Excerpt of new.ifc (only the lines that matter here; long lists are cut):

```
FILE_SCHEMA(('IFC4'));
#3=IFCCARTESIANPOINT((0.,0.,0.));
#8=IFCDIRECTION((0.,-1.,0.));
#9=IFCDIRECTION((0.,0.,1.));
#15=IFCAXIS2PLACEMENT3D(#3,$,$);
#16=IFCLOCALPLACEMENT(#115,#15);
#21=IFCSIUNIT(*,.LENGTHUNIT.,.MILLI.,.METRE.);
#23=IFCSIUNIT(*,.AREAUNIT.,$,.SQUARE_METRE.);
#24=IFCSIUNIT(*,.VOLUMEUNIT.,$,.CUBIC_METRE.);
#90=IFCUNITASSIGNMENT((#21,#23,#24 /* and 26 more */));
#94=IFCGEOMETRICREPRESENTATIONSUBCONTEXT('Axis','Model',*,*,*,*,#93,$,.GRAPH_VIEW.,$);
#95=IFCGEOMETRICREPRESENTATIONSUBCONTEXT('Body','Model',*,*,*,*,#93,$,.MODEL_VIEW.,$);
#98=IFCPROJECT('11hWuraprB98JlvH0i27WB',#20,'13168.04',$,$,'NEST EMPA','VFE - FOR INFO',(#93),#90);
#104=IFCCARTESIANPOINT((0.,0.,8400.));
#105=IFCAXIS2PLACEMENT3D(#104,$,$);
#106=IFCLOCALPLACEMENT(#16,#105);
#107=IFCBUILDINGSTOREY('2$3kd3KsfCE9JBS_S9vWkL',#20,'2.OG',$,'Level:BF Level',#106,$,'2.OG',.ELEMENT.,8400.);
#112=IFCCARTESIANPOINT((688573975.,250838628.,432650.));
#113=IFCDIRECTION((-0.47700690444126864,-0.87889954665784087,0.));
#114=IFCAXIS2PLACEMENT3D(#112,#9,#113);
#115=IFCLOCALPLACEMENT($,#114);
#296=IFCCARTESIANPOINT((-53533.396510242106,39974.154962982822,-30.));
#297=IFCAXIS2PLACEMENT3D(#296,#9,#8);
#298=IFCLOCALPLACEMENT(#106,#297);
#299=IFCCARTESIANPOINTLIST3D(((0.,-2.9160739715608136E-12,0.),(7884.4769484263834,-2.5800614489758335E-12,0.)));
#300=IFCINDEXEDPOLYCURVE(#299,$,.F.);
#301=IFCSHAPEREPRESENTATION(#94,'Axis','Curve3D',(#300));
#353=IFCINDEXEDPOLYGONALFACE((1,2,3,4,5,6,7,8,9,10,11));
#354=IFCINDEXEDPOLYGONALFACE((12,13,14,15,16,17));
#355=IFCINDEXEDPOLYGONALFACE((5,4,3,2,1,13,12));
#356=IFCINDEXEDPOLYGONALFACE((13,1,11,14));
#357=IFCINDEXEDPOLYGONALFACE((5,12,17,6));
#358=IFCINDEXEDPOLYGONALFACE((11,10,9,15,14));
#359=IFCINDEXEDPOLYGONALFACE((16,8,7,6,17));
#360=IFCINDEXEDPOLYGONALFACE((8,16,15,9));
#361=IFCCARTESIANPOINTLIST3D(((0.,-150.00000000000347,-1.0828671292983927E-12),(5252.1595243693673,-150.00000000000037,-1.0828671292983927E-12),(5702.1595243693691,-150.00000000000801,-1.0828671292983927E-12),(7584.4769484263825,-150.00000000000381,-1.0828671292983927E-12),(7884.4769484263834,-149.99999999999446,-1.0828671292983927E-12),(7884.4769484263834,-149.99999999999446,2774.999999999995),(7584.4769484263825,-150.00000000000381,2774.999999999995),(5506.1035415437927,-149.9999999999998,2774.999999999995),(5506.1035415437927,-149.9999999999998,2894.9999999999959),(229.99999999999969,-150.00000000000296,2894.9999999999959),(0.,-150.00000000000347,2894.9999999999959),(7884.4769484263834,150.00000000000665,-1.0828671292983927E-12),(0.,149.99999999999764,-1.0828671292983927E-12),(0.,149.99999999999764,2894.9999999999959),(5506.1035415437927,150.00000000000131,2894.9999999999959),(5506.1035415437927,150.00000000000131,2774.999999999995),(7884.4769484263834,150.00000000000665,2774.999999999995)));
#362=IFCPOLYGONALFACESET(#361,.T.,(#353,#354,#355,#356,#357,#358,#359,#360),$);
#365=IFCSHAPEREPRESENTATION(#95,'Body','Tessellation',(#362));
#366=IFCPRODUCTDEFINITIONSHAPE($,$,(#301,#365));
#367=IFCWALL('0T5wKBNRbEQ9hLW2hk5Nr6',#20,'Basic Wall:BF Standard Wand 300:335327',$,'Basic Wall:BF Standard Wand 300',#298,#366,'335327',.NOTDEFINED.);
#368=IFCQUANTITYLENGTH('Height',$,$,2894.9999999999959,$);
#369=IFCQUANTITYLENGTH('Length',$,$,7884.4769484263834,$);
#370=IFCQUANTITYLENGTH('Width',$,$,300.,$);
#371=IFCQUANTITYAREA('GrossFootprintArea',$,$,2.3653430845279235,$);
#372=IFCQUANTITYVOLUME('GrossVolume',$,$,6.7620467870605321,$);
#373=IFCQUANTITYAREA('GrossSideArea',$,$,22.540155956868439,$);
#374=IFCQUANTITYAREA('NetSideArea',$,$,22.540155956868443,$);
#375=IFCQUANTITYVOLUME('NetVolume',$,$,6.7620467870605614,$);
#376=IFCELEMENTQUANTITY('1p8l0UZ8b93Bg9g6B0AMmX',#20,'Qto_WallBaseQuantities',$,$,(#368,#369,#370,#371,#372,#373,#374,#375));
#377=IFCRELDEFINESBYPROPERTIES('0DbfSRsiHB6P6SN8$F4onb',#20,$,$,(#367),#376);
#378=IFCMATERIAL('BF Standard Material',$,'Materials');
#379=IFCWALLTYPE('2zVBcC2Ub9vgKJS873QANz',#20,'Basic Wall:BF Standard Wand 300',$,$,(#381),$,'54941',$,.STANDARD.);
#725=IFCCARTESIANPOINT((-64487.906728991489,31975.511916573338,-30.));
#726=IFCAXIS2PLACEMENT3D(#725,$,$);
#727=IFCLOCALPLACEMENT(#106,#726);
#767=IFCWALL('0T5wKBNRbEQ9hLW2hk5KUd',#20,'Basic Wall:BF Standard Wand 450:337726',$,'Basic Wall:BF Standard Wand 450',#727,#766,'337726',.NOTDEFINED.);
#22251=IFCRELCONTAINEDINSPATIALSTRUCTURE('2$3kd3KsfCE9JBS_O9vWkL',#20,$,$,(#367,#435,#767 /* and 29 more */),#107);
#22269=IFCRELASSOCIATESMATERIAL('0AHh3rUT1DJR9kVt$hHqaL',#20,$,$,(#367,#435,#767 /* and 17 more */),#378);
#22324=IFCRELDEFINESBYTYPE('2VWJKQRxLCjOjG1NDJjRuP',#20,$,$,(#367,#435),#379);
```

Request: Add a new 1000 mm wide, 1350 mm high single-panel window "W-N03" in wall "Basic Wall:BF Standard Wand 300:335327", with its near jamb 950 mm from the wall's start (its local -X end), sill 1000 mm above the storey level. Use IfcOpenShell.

```python
import numpy as np
import ifcopenshell
import ifcopenshell.api.feature
import ifcopenshell.api.geometry
import ifcopenshell.api.pset
import ifcopenshell.api.root
import ifcopenshell.api.spatial
import ifcopenshell.geom
import ifcopenshell.util.element
import ifcopenshell.util.placement
import ifcopenshell.util.representation
import ifcopenshell.util.shape
import ifcopenshell.util.unit

model = ifcopenshell.open("new.ifc")
unit_scale = ifcopenshell.util.unit.calculate_unit_scale(model)
area_scale = ifcopenshell.util.unit.calculate_unit_scale(model, "AREAUNIT")
volume_scale = ifcopenshell.util.unit.calculate_unit_scale(model, "VOLUMEUNIT")
settings = ifcopenshell.geom.settings()


def volume(element):
    """Net volume in cubic metres, openings subtracted."""
    shape = ifcopenshell.geom.create_shape(settings, element)
    return ifcopenshell.util.shape.get_volume(shape.geometry)


wall = model.by_guid("0T5wKBNRbEQ9hLW2hk5Nr6")
storey = ifcopenshell.util.element.get_container(wall, ifc_class="IfcBuildingStorey")
context = ifcopenshell.util.representation.get_context(model, "Model", "Body", "MODEL_VIEW")
before = volume(wall)

width, height, from_end, sill = 1, 1.35, 0.95, 1  # metres

# The wall runs along its own X axis, and the end named is its -X end.
wall_shape = ifcopenshell.geom.create_shape(settings, wall)
x, y, z = ifcopenshell.util.shape.get_vertices(wall_shape.geometry).T
start = x.min() + from_end
face, thickness = float(y.min()), float(y.max() - y.min())
wall_matrix = ifcopenshell.util.placement.get_local_placement(wall.ObjectPlacement)
level = ifcopenshell.util.placement.get_local_placement(storey.ObjectPlacement)[2, 3]


def in_wall(x, y):
    """Placement at x, y metres in the wall's axes, at sill height."""
    matrix = wall_matrix.copy()
    matrix[:, 3] = wall_matrix @ np.array([x / unit_scale, y / unit_scale, 0.0, 1.0])
    matrix[2, 3] = level + sill / unit_scale
    return matrix


# Opening: a box that overshoots both wall faces by 50 mm.
opening = ifcopenshell.api.root.create_entity(model, ifc_class="IfcOpeningElement", predefined_type="OPENING")
box = ifcopenshell.api.geometry.add_wall_representation(
    model, context=context, length=width, height=height, thickness=thickness + 0.1
)
ifcopenshell.api.geometry.assign_representation(model, product=opening, representation=box)
ifcopenshell.api.geometry.edit_object_placement(model, product=opening, matrix=in_wall(start, face - 0.05), is_si=False)
ifcopenshell.api.feature.add_feature(model, feature=opening, element=wall)

window = ifcopenshell.api.root.create_entity(model, ifc_class="IfcWindow", name="W-N03", predefined_type="WINDOW")
window.OverallWidth, window.OverallHeight = width / unit_scale, height / unit_scale
window.PartitioningType = "SINGLE_PANEL"
body = ifcopenshell.api.geometry.add_window_representation(
    model,
    context=context,
    overall_width=window.OverallWidth,
    overall_height=window.OverallHeight,
    partition_type="SINGLE_PANEL",
)
ifcopenshell.api.geometry.assign_representation(model, product=window, representation=body)
ifcopenshell.api.spatial.assign_container(model, products=[window], relating_structure=storey)
ifcopenshell.api.feature.add_filling(model, opening=opening, element=window)

# Centre the window in the wall's thickness.
ifcopenshell.api.geometry.edit_object_placement(model, product=window, matrix=in_wall(start, face), is_si=False)
window_shape = ifcopenshell.geom.create_shape(settings, window)
depth = ifcopenshell.util.shape.get_vertices(window_shape.geometry)[:, 1]
offset = face + thickness / 2 - (depth.min() + depth.max()) / 2
ifcopenshell.api.geometry.edit_object_placement(model, product=window, matrix=in_wall(start, offset), is_si=False)

after = volume(wall)

# Update the wall's stored quantities.
qto = model.by_id(ifcopenshell.util.element.get_pset(wall, "Qto_WallBaseQuantities", should_inherit=False)["id"])
ifcopenshell.api.pset.edit_qto(model, qto=qto, properties={
    "NetSideArea": after / thickness / area_scale,
    "NetVolume": after / volume_scale,
})

print(f"wall volume {before:.3f} -> {after:.3f} m3")

model.write("new_rev.ifc")
```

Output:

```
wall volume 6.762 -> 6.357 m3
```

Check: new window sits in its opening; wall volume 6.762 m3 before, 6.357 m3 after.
